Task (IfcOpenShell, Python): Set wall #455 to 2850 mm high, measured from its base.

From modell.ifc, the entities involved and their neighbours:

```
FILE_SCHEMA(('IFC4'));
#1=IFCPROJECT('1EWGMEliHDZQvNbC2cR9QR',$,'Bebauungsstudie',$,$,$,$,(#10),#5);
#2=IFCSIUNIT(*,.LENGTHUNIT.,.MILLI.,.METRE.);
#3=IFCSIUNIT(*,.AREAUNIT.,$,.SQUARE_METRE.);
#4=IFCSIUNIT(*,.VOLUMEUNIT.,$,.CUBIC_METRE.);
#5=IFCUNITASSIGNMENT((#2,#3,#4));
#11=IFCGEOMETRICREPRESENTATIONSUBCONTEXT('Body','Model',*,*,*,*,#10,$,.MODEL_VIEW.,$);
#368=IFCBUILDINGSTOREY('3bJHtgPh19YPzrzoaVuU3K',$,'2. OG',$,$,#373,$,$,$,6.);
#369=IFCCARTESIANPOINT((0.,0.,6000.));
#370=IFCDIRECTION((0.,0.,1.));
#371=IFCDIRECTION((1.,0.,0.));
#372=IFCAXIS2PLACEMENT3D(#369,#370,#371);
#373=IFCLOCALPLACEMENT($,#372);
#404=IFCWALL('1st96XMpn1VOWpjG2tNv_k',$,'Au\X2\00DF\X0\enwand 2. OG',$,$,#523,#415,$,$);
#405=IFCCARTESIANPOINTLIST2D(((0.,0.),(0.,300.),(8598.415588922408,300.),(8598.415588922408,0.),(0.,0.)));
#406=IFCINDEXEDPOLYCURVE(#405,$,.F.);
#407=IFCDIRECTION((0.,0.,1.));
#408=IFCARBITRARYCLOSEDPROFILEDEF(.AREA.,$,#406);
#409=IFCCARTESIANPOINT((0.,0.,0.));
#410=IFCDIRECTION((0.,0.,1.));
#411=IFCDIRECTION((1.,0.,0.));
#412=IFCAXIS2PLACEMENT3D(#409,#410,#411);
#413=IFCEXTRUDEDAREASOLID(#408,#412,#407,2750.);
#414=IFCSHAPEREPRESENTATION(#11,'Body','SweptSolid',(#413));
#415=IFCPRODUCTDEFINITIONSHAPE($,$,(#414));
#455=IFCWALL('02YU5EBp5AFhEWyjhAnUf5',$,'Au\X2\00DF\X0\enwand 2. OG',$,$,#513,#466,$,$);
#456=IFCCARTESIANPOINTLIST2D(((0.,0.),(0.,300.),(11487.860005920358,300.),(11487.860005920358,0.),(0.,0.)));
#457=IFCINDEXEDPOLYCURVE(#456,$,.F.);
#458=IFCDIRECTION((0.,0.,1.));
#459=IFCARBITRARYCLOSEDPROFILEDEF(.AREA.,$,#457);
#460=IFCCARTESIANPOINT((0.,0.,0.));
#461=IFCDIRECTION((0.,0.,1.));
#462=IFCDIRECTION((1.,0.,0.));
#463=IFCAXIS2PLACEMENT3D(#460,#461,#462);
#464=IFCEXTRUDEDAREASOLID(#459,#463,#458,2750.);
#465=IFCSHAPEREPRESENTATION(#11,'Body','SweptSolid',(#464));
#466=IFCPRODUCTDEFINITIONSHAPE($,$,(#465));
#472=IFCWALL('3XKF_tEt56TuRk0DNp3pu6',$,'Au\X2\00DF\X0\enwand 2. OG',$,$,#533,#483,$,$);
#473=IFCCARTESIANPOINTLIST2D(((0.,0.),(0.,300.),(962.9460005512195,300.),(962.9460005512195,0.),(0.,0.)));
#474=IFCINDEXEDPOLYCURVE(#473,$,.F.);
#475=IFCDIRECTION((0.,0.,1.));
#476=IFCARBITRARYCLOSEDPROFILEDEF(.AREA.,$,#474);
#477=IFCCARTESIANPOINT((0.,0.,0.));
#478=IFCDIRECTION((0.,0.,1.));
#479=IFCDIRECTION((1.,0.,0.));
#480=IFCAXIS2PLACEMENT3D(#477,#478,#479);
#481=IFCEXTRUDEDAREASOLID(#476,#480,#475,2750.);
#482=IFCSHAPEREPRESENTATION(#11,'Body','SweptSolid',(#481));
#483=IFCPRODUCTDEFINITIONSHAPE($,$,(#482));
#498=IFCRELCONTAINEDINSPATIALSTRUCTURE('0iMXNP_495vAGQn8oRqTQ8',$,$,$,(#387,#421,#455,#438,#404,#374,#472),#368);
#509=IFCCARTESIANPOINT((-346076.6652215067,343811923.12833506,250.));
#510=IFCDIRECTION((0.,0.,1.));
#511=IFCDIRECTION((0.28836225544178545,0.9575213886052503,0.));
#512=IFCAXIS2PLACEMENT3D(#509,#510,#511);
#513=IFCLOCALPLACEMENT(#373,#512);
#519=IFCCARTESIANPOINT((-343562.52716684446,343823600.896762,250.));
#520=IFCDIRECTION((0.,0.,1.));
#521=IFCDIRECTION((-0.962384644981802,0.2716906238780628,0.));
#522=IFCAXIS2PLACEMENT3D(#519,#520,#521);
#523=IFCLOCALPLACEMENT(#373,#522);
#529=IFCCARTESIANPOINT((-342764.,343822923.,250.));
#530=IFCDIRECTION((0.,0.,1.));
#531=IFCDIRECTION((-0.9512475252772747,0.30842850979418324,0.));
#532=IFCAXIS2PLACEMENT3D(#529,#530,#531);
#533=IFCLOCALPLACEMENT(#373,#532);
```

```python
import ifcopenshell
import ifcopenshell.geom
import ifcopenshell.util.representation
import ifcopenshell.util.shape

model = ifcopenshell.open("modell.ifc")
settings = ifcopenshell.geom.settings()


def volume(element):
    """Net volume in cubic metres, openings subtracted."""
    shape = ifcopenshell.geom.create_shape(settings, element)
    return ifcopenshell.util.shape.get_volume(shape.geometry)


wall = model.by_guid("02YU5EBp5AFhEWyjhAnUf5")
before = volume(wall)

body = ifcopenshell.util.representation.get_representation(wall, "Model", "Body")
solid = body.Items[0]
old_height = solid.Depth
solid.Depth = 2850.0
after = volume(wall)

print(f"height {old_height:g} -> {solid.Depth:g}, volume {before:.3f} -> {after:.3f} m3")

model.write("modell-out.ifc")
```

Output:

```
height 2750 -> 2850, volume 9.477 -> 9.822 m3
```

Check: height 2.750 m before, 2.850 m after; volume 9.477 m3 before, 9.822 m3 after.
